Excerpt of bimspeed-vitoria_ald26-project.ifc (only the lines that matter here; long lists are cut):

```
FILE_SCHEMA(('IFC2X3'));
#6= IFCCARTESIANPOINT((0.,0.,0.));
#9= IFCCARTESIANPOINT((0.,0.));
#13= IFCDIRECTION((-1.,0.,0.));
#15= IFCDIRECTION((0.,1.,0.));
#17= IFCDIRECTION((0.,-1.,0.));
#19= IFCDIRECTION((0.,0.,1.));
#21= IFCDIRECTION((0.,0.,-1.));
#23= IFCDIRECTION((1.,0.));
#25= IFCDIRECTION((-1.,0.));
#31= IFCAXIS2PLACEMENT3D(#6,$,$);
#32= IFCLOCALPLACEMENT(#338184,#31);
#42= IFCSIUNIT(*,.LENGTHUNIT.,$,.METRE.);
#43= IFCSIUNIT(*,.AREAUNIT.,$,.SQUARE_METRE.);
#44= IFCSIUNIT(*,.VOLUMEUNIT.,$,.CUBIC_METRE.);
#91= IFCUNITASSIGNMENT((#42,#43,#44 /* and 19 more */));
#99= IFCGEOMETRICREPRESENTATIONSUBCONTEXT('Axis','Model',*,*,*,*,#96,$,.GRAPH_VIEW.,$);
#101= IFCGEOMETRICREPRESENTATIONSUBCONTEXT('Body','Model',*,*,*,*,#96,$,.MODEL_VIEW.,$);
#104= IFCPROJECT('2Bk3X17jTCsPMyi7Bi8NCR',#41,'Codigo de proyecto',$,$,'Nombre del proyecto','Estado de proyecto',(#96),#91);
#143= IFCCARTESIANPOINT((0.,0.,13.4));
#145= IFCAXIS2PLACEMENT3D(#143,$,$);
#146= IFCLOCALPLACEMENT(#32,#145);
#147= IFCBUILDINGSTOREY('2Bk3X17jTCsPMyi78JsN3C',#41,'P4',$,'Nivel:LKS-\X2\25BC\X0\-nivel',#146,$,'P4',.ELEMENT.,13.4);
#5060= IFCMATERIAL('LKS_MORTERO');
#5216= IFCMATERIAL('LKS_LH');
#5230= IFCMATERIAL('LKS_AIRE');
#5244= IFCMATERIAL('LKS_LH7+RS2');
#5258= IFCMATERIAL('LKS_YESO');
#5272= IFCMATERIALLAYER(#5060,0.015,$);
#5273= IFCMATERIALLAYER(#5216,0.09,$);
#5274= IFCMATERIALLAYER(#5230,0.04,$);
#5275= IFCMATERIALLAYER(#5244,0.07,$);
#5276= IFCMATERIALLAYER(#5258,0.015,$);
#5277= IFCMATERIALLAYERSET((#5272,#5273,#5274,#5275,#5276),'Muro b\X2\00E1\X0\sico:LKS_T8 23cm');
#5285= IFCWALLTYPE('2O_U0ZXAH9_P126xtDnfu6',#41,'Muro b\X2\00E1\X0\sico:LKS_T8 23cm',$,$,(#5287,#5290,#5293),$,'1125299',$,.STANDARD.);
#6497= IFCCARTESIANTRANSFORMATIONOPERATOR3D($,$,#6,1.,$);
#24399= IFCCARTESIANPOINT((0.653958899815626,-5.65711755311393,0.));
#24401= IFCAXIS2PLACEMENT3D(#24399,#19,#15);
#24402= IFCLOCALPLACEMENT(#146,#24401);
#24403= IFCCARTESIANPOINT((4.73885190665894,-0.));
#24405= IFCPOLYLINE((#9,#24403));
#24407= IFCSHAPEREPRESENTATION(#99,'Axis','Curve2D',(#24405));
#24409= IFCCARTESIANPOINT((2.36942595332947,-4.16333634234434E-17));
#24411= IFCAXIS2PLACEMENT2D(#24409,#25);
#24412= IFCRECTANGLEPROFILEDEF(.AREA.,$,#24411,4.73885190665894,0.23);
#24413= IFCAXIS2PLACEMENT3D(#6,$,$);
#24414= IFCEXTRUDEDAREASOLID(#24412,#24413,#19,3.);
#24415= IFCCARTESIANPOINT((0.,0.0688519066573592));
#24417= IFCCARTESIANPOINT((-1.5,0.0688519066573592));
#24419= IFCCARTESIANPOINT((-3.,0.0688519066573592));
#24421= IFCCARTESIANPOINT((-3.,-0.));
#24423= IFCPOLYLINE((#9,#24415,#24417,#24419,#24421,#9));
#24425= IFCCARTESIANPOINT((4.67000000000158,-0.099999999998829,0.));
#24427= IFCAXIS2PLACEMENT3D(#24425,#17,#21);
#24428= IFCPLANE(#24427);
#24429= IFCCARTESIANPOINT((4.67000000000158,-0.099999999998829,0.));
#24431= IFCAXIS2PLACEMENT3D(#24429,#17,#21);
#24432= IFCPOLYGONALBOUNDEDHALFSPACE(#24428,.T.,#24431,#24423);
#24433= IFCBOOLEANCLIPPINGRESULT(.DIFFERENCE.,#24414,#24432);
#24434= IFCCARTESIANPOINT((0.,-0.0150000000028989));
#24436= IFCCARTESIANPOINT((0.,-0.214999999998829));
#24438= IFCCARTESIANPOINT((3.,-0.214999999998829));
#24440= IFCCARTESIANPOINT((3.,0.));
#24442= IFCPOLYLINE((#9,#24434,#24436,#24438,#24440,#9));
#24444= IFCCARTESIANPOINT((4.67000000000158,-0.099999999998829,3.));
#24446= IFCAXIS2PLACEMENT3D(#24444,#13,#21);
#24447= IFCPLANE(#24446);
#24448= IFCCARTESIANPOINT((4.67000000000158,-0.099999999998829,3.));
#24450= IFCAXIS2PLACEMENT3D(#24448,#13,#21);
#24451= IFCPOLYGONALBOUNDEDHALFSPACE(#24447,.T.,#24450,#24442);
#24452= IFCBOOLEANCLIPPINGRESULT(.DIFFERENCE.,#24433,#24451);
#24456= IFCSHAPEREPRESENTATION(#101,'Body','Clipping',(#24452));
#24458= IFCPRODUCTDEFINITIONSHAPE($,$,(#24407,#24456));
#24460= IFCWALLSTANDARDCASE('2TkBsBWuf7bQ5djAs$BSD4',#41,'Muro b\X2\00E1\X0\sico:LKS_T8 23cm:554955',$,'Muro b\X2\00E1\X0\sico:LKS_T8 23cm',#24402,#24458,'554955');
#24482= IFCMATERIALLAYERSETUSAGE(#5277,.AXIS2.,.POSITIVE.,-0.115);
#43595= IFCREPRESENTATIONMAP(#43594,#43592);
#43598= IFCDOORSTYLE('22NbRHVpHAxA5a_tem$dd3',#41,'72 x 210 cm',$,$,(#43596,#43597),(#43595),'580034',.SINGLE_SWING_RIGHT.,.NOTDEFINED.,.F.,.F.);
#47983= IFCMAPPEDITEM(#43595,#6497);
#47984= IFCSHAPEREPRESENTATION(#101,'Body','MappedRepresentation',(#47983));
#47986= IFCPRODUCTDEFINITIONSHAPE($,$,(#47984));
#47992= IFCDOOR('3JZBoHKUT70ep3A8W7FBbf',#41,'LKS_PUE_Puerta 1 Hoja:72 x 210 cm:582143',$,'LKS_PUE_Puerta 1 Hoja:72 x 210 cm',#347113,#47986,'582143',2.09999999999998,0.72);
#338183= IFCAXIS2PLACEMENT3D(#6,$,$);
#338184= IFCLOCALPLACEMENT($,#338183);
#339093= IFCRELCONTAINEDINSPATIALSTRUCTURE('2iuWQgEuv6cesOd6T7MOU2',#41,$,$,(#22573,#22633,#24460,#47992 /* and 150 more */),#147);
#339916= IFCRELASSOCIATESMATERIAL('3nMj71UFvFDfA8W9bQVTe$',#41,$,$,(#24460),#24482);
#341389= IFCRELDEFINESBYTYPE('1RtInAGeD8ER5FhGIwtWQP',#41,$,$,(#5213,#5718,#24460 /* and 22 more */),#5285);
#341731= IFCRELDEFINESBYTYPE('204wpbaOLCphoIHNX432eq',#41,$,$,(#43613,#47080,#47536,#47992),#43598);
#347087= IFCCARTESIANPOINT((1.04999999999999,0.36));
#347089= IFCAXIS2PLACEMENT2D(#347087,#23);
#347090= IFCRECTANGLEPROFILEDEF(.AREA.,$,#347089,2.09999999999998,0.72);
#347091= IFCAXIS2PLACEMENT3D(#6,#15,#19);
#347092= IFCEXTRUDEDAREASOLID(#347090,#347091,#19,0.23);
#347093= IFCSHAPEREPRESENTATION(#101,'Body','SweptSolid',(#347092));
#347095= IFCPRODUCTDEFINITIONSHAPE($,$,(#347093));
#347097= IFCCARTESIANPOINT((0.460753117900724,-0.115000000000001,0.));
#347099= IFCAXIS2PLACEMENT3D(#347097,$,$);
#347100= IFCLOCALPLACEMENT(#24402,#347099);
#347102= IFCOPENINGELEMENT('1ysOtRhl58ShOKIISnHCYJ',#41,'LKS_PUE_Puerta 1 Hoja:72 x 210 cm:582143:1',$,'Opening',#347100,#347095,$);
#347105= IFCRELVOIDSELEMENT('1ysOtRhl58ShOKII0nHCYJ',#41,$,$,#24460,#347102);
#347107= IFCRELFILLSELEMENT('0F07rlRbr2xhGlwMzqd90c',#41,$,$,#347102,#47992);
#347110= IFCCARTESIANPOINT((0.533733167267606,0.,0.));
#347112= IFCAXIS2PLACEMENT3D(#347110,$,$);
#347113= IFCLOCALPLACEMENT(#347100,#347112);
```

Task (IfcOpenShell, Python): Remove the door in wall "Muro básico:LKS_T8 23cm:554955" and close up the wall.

```python
import ifcopenshell
import ifcopenshell.api.feature
import ifcopenshell.api.root
import ifcopenshell.geom
import ifcopenshell.util.shape

model = ifcopenshell.open("bimspeed-vitoria_ald26-project.ifc")
settings = ifcopenshell.geom.settings()


def volume(element):
    """Net volume in cubic metres, openings subtracted."""
    shape = ifcopenshell.geom.create_shape(settings, element)
    return ifcopenshell.util.shape.get_volume(shape.geometry)


door = model.by_guid("3JZBoHKUT70ep3A8W7FBbf")
opening = door.FillsVoids[0].RelatingOpeningElement
wall = opening.VoidsElements[0].RelatingBuildingElement
before = volume(wall)

ifcopenshell.api.root.remove_product(model, product=door)
ifcopenshell.api.feature.remove_feature(model, feature=opening)

after = volume(wall)

print(f"wall volume {before:.3f} -> {after:.3f} m3")

model.write("bimspeed-vitoria_ald26-project_rev.ifc")
```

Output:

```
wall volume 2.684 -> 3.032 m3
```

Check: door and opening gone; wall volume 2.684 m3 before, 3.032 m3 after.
